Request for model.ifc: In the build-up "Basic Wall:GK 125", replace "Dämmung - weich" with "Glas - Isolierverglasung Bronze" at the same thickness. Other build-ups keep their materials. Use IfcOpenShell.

First a look at what the model holds.

```python
import ifcopenshell
import ifcopenshell.util.element

model = ifcopenshell.open("model.ifc")
print(model.schema)
for layer_set in model.by_type("IfcMaterialLayerSet"):
    if layer_set.LayerSetName == "Basic Wall:GK 125":
        for layer in layer_set.MaterialLayers:
            print(layer.id(), layer.Material and layer.Material.Name, layer.LayerThickness, sep=" | ")
        print(len(ifcopenshell.util.element.get_elements_by_material(model, layer_set)), "elements and types use it")
print(sorted(m.Name for m in model.by_type("IfcMaterial") if m.Name)[:60])
```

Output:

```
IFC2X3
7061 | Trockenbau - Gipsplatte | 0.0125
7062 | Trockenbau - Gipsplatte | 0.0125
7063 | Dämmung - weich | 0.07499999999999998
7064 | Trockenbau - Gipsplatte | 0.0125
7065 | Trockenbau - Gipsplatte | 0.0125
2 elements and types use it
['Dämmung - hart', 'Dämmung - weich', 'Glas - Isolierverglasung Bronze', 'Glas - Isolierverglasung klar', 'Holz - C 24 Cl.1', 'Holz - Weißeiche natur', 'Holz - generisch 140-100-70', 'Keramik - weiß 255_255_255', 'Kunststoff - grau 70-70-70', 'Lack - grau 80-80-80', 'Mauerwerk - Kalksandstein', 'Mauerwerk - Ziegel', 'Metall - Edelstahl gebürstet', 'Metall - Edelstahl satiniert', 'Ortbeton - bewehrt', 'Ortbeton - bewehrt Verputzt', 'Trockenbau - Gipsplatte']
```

```python
import ifcopenshell
import ifcopenshell.api.material

model = ifcopenshell.open("model.ifc")

layer_set = next(s for s in model.by_type("IfcMaterialLayerSet") if s.LayerSetName == "Basic Wall:GK 125")
layer = next(l for l in layer_set.MaterialLayers if l.Material and l.Material.Name == "Dämmung - weich")
material = next(m for m in model.by_type("IfcMaterial") if m.Name == "Glas - Isolierverglasung Bronze")

# Point this one layer at the other material; renaming the old one would change it everywhere.
ifcopenshell.api.material.edit_layer(model, layer=layer, attributes={}, material=material)

print([l.Material.Name if l.Material else None for l in layer_set.MaterialLayers])

model.write("model_v2.ifc")
```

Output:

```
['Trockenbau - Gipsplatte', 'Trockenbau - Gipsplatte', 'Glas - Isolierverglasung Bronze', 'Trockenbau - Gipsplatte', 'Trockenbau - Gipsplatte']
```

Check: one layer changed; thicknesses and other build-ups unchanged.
